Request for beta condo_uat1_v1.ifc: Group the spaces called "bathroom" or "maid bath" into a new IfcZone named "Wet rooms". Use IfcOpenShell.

First a look at what the model holds.

```python
import ifcopenshell

model = ifcopenshell.open("beta condo_uat1_v1.ifc")
print(model.schema)
seen = {}
for space in model.by_type("IfcSpace"):
    seen[space.LongName] = seen.get(space.LongName, 0) + 1
for name, count in sorted(seen.items(), key=str):
    print(count, "x", name)
print("zones:", [z.Name for z in model.by_type("IfcZone")][:20])
```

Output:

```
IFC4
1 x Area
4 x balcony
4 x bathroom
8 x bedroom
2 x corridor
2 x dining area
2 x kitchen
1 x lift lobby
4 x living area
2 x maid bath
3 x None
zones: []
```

```python
import ifcopenshell
import ifcopenshell.api.group
import ifcopenshell.api.root

model = ifcopenshell.open("beta condo_uat1_v1.ifc")

names = {"bathroom", "maid bath"}
spaces = [s for s in model.by_type("IfcSpace") if s.LongName in names]

zone = ifcopenshell.api.root.create_entity(model, ifc_class="IfcZone", name="Wet rooms")
ifcopenshell.api.group.assign_group(model, products=spaces, group=zone)
print(len(spaces), "spaces in", zone.Name)

model.write("beta condo_uat1_v1_updated.ifc")
```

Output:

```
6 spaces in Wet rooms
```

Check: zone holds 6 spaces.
